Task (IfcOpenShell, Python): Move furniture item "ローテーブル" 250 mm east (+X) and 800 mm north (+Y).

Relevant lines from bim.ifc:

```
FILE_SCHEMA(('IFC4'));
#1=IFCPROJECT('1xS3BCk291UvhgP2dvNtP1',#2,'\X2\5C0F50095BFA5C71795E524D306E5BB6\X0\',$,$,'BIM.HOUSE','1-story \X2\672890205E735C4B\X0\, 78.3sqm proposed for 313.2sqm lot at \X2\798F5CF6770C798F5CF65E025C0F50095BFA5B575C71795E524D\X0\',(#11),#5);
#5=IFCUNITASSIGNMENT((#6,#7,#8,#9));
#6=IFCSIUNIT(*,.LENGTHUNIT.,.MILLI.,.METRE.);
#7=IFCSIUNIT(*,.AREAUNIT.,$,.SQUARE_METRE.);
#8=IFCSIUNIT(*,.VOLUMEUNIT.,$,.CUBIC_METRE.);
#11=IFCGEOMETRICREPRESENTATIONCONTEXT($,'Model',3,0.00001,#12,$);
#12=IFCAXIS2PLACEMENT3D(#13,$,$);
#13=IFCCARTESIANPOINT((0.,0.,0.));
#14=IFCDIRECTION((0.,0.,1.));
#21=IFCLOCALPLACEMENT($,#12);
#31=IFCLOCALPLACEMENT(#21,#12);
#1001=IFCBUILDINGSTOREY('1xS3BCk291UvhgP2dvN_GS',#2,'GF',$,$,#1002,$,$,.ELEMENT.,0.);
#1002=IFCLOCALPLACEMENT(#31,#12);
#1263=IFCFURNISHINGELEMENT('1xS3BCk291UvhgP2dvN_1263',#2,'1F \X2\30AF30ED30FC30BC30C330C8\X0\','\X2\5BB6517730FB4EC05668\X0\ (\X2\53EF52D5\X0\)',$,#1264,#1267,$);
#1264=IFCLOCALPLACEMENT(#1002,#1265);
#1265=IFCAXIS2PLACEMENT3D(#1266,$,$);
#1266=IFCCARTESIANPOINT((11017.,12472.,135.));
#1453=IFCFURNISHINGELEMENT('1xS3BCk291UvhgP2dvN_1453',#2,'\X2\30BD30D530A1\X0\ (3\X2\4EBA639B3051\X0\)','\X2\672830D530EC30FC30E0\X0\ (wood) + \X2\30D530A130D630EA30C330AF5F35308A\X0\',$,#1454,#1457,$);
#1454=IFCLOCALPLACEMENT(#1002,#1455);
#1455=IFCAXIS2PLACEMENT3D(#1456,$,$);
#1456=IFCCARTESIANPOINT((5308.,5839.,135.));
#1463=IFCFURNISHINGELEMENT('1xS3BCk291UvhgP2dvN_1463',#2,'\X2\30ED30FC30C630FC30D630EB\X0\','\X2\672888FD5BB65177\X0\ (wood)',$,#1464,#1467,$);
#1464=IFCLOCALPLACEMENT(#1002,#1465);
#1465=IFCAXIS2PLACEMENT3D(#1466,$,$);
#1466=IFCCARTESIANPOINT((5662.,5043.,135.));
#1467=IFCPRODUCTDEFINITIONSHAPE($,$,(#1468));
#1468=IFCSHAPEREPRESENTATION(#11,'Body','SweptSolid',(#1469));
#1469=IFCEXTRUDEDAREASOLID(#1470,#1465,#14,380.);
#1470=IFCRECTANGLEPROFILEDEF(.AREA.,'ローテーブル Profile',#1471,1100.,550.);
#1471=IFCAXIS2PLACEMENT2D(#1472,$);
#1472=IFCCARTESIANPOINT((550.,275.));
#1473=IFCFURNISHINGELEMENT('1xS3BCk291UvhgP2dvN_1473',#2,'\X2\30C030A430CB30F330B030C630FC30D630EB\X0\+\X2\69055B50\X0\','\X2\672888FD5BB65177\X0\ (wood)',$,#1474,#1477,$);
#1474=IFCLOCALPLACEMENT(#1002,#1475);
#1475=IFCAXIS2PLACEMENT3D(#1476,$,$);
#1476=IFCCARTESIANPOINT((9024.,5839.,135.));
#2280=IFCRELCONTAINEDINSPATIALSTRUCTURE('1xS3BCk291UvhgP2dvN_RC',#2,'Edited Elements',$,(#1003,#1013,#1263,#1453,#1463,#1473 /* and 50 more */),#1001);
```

```python
import ifcopenshell
import ifcopenshell.api.geometry
import ifcopenshell.util.placement
import ifcopenshell.util.unit

model = ifcopenshell.open("bim.ifc")
unit_scale = ifcopenshell.util.unit.calculate_unit_scale(model)

item = model.by_guid("1xS3BCk291UvhgP2dvN_1463")
matrix = ifcopenshell.util.placement.get_local_placement(item.ObjectPlacement)
matrix[0, 3] += 0.25 / unit_scale
matrix[1, 3] += 0.8 / unit_scale
ifcopenshell.api.geometry.edit_object_placement(model, product=item, matrix=matrix, is_si=False)

print(ifcopenshell.util.placement.get_local_placement(item.ObjectPlacement).round(3) + 0.0)

model.write("bim_v2.ifc")
```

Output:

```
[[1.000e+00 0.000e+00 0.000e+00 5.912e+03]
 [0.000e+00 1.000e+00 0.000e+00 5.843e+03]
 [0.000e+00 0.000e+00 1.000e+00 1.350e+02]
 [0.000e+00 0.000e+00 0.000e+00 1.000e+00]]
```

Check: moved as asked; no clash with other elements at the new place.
